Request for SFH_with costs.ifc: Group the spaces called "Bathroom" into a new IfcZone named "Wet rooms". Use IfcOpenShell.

First a look at what the model holds.

```python
import ifcopenshell

model = ifcopenshell.open("SFH_with costs.ifc")
print(model.schema)
seen = {}
for space in model.by_type("IfcSpace"):
    seen[space.LongName] = seen.get(space.LongName, 0) + 1
for name, count in sorted(seen.items(), key=str):
    print(count, "x", name)
print("zones:", [z.Name for z in model.by_type("IfcZone")][:20])
```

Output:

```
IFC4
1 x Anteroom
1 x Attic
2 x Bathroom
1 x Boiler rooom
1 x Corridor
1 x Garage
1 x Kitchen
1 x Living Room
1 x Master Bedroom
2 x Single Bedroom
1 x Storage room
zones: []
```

```python
import ifcopenshell
import ifcopenshell.api.group
import ifcopenshell.api.root

model = ifcopenshell.open("SFH_with costs.ifc")

names = {"Bathroom"}
spaces = [s for s in model.by_type("IfcSpace") if s.LongName in names]

zone = ifcopenshell.api.root.create_entity(model, ifc_class="IfcZone", name="Wet rooms")
ifcopenshell.api.group.assign_group(model, products=spaces, group=zone)
print(len(spaces), "spaces in", zone.Name)

model.write("SFH_with costs_updated.ifc")
```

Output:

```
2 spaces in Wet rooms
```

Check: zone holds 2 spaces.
